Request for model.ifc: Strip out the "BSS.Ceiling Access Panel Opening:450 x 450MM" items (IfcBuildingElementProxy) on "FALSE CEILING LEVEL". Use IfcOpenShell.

First a look at what the model holds.

```python
import ifcopenshell
import ifcopenshell.util.element

model = ifcopenshell.open("model.ifc")
print(model.schema)
storey = next(s for s in model.by_type("IfcBuildingStorey") if s.Name == "FALSE CEILING LEVEL")
proxies = [e for e in ifcopenshell.util.element.get_decomposition(storey) if e.is_a("IfcBuildingElementProxy")]
seen = {}
for e in proxies:
    element_type = ifcopenshell.util.element.get_type(e)
    name = element_type.Name if element_type not in (None, e) else None
    seen[name] = seen.get(name, 0) + 1
for name, count in sorted(seen.items(), key=str):
    print(count, "x", name)
```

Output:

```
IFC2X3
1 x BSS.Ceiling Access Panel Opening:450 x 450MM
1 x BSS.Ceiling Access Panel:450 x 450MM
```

```python
import ifcopenshell
import ifcopenshell.api.root
import ifcopenshell.util.element

model = ifcopenshell.open("model.ifc")

storey = next(s for s in model.by_type("IfcBuildingStorey") if s.Name == "FALSE CEILING LEVEL")
proxies = [e for e in ifcopenshell.util.element.get_decomposition(storey) if e.is_a("IfcBuildingElementProxy")]
targets = [e for e in proxies if (t := ifcopenshell.util.element.get_type(e)) not in (None, e) and t.Name == "BSS.Ceiling Access Panel Opening:450 x 450MM"]

for e in targets:
    ifcopenshell.api.root.remove_product(model, product=e)
print(len(targets), "removed")

model.write("model_v2.ifc")
```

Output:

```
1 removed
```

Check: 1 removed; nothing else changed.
